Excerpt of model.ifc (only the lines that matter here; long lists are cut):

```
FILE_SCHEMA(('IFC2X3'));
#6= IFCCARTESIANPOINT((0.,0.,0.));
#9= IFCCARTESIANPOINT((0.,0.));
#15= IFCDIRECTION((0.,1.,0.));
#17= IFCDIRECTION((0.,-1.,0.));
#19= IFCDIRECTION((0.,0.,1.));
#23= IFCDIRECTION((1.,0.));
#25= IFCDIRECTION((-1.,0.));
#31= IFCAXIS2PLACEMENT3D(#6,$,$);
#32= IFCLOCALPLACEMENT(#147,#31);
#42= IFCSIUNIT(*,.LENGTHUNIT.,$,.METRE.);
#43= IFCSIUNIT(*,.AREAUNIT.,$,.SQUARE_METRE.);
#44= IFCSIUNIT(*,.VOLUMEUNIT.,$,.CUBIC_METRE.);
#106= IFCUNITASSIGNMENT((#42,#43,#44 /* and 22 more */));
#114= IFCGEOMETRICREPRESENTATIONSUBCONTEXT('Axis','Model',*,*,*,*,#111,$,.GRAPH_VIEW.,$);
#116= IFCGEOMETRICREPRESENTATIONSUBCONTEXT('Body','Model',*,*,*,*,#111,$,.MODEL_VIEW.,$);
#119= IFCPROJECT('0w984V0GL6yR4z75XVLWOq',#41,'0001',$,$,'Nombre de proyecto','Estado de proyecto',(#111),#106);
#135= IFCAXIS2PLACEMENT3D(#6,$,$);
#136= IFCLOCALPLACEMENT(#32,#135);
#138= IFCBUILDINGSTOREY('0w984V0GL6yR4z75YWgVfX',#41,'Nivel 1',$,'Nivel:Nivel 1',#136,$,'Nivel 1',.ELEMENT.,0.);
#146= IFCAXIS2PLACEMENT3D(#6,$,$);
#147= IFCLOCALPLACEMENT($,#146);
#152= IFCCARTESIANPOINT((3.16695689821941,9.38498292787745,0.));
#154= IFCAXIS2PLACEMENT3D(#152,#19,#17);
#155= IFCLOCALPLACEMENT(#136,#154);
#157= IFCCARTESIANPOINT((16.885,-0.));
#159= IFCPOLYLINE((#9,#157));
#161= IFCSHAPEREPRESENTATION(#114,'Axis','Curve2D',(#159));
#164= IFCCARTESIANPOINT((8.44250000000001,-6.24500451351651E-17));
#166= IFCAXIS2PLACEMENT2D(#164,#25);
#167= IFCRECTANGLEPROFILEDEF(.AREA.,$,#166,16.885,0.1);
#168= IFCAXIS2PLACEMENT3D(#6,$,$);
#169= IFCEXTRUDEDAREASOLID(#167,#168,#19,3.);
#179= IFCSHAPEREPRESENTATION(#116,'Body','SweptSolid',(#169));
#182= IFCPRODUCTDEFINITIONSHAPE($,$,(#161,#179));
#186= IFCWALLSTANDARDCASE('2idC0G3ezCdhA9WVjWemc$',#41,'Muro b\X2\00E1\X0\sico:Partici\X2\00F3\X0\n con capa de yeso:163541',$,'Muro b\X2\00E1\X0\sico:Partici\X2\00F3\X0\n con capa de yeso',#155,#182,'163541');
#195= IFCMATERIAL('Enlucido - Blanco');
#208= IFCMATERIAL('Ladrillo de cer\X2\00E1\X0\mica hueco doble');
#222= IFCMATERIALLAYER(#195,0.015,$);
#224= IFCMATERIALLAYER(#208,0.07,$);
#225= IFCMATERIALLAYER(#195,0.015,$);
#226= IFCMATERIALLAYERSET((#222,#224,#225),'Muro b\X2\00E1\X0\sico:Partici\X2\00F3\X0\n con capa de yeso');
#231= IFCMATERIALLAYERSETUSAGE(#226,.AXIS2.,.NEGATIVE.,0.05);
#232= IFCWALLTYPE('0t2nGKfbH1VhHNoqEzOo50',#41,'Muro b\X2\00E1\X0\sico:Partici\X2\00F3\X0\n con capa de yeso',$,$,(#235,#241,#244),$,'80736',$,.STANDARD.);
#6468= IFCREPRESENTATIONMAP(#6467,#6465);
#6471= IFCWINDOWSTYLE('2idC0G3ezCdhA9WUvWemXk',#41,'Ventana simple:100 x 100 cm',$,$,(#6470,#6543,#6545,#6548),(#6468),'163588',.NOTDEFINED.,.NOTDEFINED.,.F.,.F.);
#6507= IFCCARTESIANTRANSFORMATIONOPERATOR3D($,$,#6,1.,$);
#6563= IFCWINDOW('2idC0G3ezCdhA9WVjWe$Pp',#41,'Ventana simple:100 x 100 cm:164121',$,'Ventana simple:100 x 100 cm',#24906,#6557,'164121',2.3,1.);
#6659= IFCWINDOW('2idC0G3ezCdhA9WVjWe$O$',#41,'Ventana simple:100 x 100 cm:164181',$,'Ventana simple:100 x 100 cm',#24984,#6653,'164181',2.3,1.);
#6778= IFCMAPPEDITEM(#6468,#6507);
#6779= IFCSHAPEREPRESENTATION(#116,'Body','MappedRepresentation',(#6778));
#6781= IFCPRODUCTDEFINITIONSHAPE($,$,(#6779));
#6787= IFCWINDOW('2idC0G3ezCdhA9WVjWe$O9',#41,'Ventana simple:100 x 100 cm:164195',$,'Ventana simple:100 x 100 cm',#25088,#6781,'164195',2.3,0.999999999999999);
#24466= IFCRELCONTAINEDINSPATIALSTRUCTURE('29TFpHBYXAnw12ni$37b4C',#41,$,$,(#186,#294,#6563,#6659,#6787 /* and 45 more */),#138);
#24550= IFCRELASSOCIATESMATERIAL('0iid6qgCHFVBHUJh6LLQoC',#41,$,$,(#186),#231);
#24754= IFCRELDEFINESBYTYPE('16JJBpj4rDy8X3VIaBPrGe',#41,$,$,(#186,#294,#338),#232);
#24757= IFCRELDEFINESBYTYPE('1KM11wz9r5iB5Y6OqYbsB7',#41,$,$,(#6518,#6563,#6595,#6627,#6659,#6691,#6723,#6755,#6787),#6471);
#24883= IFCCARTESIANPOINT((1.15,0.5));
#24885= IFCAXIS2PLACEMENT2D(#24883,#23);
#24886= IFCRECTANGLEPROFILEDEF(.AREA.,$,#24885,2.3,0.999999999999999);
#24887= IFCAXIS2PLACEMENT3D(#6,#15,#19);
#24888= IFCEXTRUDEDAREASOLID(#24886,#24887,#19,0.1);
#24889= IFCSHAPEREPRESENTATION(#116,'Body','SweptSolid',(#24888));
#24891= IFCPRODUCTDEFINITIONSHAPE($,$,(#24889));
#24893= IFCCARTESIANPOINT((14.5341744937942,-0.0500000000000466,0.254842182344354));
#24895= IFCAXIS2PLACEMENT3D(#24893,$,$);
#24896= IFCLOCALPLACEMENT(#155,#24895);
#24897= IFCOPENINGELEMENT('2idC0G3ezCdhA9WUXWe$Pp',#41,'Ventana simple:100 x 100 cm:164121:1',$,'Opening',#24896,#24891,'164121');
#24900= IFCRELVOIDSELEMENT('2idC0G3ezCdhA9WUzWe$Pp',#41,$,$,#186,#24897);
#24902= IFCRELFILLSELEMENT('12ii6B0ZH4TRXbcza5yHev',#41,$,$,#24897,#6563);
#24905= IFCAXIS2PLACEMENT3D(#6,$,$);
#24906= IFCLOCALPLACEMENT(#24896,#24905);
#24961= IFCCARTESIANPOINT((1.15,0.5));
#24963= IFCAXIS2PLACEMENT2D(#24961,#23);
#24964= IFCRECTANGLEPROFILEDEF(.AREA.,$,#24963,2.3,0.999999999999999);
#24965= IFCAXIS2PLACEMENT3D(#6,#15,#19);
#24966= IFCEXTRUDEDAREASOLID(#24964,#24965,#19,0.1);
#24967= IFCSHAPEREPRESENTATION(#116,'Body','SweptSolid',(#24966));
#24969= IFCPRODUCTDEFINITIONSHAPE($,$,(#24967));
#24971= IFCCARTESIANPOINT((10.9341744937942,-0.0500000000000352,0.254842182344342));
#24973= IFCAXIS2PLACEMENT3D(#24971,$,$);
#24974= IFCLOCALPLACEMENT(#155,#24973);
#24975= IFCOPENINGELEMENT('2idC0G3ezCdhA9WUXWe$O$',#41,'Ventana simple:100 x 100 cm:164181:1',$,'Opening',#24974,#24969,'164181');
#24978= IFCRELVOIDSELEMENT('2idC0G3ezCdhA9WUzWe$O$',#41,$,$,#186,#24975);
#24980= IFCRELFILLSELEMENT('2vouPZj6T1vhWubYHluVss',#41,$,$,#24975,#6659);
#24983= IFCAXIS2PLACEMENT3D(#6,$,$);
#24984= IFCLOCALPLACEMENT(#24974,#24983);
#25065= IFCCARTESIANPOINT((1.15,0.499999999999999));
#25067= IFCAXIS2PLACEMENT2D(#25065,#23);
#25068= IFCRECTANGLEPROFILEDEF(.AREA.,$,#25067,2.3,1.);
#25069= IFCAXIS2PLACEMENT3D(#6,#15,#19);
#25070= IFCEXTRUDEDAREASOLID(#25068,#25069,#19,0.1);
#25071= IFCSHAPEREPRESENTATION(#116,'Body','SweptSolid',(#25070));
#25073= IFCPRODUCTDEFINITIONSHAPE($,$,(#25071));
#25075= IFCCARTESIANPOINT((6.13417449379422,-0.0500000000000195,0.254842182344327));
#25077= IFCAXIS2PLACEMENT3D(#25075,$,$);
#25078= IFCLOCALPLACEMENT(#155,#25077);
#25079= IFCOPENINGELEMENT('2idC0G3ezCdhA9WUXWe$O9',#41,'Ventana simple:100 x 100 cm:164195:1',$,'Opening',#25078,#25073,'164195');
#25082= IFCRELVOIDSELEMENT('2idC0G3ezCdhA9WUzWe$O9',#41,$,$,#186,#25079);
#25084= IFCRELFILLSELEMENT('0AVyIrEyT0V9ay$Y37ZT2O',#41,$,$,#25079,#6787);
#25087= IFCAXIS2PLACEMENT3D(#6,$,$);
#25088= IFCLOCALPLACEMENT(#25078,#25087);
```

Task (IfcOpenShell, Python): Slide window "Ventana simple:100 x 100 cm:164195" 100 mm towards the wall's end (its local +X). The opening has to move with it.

```python
import ifcopenshell
import ifcopenshell.api.geometry
import ifcopenshell.util.placement

model = ifcopenshell.open("model.ifc")

window = model.by_guid("2idC0G3ezCdhA9WVjWe$O9")
opening = window.FillsVoids[0].RelatingOpeningElement
wall = opening.VoidsElements[0].RelatingBuildingElement

wall_matrix = ifcopenshell.util.placement.get_local_placement(wall.ObjectPlacement)
shift = wall_matrix[:3, 0] * 0.1
before = ifcopenshell.util.placement.get_local_placement(window.ObjectPlacement)[:3, 3].copy()

# The window is placed relative to its opening, so it follows when the opening moves.
matrix = ifcopenshell.util.placement.get_local_placement(opening.ObjectPlacement)
matrix[:3, 3] += shift
ifcopenshell.api.geometry.edit_object_placement(
    model, product=opening, matrix=matrix, is_si=False, should_transform_children=True
)

after = ifcopenshell.util.placement.get_local_placement(window.ObjectPlacement)[:3, 3]
print("window moved by", (after - before).round(3) + 0.0)

model.write("model_updated.ifc")
```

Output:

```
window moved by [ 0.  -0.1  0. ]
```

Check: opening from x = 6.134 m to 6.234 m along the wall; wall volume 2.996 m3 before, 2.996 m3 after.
